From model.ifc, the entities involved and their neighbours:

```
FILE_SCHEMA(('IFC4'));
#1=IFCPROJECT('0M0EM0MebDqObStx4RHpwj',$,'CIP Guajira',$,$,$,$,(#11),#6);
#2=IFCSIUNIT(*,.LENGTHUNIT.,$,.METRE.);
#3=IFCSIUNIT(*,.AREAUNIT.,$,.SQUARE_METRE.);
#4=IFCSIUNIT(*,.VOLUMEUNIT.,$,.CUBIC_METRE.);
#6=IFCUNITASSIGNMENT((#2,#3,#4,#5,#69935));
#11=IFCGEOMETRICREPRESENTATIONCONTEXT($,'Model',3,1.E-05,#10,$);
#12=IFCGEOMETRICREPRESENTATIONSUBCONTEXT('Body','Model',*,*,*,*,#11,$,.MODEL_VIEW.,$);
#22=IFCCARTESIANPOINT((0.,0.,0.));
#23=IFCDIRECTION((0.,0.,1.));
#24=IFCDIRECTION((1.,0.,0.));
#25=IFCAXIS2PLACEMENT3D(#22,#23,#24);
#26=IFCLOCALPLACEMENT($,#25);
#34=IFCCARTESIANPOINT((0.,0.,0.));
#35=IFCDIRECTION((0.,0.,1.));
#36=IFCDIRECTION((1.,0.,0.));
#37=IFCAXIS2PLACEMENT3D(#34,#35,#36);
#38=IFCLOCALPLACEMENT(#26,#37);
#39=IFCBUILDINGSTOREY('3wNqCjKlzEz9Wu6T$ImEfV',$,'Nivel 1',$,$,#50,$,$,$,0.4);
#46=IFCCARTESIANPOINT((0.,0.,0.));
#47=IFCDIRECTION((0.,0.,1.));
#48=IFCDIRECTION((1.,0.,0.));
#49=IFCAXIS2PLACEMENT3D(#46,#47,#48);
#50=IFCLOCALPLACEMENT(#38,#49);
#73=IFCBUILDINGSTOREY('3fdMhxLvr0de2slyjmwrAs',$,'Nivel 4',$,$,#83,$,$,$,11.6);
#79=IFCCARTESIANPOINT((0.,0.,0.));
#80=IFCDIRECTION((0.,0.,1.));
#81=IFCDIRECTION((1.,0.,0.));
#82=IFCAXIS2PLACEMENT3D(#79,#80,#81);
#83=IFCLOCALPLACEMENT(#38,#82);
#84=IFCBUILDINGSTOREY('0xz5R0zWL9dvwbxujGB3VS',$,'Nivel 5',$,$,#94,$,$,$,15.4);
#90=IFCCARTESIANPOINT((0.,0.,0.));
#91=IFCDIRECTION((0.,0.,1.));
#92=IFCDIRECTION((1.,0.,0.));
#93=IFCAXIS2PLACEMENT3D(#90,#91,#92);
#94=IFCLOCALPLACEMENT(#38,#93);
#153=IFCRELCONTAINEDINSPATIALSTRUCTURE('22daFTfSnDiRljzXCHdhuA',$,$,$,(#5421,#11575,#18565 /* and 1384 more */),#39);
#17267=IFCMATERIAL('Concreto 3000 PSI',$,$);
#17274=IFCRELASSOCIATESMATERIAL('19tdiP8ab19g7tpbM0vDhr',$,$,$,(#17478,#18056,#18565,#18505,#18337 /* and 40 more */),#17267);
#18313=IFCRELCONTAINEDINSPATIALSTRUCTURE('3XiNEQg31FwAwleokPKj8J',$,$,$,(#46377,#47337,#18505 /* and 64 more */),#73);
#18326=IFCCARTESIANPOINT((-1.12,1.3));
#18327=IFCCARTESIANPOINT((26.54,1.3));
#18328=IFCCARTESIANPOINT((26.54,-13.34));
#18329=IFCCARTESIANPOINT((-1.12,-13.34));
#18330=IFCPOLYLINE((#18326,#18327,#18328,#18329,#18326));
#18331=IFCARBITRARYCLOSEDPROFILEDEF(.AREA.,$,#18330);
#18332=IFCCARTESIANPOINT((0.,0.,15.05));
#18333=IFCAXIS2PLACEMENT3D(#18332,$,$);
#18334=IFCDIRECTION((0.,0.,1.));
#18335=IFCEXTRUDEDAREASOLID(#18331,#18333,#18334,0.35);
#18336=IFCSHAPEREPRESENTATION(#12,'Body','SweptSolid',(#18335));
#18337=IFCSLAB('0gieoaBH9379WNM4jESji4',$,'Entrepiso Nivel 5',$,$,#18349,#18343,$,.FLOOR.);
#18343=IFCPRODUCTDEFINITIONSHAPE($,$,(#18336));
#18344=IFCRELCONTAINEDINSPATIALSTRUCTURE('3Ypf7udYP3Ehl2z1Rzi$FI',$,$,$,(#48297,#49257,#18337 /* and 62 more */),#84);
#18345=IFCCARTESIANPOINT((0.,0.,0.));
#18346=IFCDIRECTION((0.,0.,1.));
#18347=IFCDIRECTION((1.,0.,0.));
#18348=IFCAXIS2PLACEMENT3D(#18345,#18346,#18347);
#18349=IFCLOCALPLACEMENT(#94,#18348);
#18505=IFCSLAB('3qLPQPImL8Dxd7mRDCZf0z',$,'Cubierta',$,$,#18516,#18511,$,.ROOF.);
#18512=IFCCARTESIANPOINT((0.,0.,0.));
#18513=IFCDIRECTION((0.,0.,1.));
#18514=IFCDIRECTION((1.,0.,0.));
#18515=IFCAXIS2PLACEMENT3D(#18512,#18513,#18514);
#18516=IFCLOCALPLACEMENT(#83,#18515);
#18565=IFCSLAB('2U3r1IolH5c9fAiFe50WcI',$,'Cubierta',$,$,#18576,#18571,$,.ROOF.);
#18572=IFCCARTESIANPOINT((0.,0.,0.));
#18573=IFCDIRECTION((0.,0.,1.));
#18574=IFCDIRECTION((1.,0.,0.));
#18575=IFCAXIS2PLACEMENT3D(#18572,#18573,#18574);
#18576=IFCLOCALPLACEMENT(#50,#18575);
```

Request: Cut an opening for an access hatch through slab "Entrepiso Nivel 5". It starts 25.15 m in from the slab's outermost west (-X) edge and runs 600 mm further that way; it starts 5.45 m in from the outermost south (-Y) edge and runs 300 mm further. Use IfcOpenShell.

```python
import numpy as np
import ifcopenshell
import ifcopenshell.api.feature
import ifcopenshell.api.geometry
import ifcopenshell.api.root
import ifcopenshell.geom
import ifcopenshell.util.placement
import ifcopenshell.util.representation
import ifcopenshell.util.shape
import ifcopenshell.util.unit

model = ifcopenshell.open("model.ifc")
unit_scale = ifcopenshell.util.unit.calculate_unit_scale(model)
settings = ifcopenshell.geom.settings()


def volume(element):
    """Net volume in cubic metres, openings subtracted."""
    shape = ifcopenshell.geom.create_shape(settings, element)
    return ifcopenshell.util.shape.get_volume(shape.geometry)


slab = model.by_guid("0gieoaBH9379WNM4jESji4")
before = volume(slab)

# Extent in the slab's own axes, in metres. The edges named are its -X and -Y sides.
slab_shape = ifcopenshell.geom.create_shape(settings, slab)
vertices = ifcopenshell.util.shape.get_vertices(slab_shape.geometry)
x_min, y_min, bottom = vertices.min(axis=0)
top = vertices[:, 2].max()

opening = ifcopenshell.api.root.create_entity(model, ifc_class="IfcOpeningElement", name="Access hatch opening", predefined_type="OPENING")
context = ifcopenshell.util.representation.get_context(model, "Model", "Body", "MODEL_VIEW")
width, depth = 0.6, 0.3
outline = [(0.0, 0.0), (width, 0.0), (width, depth), (0.0, depth), (0.0, 0.0)]
# Overshoot both faces by 50 mm so the cut is clean.
shape = ifcopenshell.api.geometry.add_slab_representation(
    model, context=context, depth=top - bottom + 0.1, polyline=outline
)
ifcopenshell.api.geometry.assign_representation(model, product=opening, representation=shape)

matrix = ifcopenshell.util.placement.get_local_placement(slab.ObjectPlacement)
matrix[:, 3] = matrix @ np.append(np.array([x_min + 25.15, y_min + 5.45, bottom - 0.05]) / unit_scale, 1.0)
ifcopenshell.api.geometry.edit_object_placement(model, product=opening, matrix=matrix, is_si=False)
ifcopenshell.api.feature.add_feature(model, feature=opening, element=slab)

after = volume(slab)

print(f"slab volume {before:.3f} -> {after:.3f} m3")

model.write("model_edited.ifc")
```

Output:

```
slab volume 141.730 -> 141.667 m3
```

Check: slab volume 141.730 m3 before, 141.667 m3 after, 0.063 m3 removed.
